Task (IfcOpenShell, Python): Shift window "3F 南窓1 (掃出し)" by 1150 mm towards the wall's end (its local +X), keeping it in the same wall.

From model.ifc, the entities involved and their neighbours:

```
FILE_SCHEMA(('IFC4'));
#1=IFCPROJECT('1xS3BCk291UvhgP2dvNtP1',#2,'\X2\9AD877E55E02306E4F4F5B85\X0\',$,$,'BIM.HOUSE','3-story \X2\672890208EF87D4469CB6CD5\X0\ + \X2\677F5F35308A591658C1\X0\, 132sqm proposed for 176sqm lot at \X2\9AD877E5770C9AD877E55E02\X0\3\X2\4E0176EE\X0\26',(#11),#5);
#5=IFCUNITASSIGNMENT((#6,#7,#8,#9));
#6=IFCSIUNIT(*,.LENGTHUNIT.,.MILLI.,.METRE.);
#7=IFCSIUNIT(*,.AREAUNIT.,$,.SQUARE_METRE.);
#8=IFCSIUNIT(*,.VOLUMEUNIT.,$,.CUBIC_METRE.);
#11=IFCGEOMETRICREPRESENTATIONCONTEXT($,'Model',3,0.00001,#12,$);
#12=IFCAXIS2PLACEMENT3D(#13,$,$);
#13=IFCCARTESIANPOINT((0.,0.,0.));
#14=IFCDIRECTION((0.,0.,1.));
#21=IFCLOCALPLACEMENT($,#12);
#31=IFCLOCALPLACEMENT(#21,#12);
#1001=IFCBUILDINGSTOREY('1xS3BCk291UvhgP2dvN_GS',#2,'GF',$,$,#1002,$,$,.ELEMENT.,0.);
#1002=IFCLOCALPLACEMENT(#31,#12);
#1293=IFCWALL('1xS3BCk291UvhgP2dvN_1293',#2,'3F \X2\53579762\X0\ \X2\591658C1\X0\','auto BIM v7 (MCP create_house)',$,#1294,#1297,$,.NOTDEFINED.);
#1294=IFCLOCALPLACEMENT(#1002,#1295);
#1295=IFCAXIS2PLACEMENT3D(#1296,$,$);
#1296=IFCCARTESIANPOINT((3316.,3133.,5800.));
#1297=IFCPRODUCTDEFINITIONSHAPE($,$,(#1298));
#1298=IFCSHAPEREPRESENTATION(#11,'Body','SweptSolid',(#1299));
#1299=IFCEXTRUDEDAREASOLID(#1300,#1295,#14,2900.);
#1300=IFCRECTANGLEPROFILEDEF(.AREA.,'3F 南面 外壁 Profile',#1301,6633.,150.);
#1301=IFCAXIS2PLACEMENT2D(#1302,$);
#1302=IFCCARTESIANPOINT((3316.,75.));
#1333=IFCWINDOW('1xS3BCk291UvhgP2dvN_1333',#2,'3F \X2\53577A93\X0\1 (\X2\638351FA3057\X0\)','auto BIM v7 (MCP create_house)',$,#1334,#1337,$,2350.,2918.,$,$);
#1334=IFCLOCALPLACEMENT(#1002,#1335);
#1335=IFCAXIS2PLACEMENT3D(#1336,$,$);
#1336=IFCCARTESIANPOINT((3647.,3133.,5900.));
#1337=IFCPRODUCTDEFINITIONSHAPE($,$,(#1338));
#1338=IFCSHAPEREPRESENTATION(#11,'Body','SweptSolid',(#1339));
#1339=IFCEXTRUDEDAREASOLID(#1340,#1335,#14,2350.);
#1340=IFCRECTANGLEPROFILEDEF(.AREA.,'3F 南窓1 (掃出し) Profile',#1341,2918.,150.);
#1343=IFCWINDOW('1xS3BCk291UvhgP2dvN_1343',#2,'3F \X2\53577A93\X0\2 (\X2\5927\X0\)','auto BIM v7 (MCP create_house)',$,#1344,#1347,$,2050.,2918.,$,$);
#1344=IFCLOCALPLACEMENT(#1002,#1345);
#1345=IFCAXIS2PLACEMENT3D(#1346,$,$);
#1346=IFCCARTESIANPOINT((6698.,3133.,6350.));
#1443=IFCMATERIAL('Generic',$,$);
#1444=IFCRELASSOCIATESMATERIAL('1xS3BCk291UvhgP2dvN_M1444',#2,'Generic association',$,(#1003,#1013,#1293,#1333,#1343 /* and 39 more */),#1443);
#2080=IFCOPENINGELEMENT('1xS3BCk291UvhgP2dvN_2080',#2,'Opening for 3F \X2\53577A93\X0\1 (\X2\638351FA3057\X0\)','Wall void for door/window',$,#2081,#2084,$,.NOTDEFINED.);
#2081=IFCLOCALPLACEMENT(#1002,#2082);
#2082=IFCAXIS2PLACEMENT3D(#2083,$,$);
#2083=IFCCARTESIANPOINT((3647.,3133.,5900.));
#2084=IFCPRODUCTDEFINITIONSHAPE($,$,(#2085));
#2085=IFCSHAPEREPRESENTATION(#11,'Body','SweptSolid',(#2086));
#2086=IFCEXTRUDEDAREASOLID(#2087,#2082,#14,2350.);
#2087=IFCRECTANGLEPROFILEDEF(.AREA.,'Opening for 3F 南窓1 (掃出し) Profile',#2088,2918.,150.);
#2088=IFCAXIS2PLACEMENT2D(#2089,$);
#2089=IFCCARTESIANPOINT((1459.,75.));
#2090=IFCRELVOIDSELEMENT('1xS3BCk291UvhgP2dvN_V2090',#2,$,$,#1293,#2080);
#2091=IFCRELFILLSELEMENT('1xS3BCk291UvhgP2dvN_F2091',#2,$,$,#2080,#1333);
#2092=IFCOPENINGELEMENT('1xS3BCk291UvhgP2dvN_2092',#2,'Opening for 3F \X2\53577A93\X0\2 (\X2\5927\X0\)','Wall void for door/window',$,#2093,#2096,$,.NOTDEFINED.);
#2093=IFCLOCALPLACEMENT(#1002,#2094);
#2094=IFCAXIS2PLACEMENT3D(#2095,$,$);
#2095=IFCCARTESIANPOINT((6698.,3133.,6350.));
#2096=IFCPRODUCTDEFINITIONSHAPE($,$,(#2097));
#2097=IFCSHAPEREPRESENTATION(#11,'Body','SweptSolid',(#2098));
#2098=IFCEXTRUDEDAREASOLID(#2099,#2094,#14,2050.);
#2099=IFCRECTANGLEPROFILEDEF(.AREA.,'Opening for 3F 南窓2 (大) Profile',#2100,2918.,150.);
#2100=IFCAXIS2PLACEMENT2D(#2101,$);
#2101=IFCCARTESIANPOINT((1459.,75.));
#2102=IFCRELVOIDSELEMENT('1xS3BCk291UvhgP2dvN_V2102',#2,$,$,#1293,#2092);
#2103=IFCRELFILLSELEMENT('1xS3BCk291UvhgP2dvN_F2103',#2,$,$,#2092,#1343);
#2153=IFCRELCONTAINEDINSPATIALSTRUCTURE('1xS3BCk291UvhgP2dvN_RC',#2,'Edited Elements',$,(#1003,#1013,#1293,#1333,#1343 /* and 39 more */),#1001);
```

```python
import ifcopenshell
import ifcopenshell.api.geometry
import ifcopenshell.util.placement
import ifcopenshell.util.unit

model = ifcopenshell.open("model.ifc")
unit_scale = ifcopenshell.util.unit.calculate_unit_scale(model)

window = model.by_guid("1xS3BCk291UvhgP2dvN_1333")
opening = window.FillsVoids[0].RelatingOpeningElement
wall = opening.VoidsElements[0].RelatingBuildingElement

wall_matrix = ifcopenshell.util.placement.get_local_placement(wall.ObjectPlacement)
shift = wall_matrix[:3, 0] * 1.15 / unit_scale
before = ifcopenshell.util.placement.get_local_placement(window.ObjectPlacement)[:3, 3].copy()

# The window is not placed relative to its opening, so move both.
for product in (opening, window):
    matrix = ifcopenshell.util.placement.get_local_placement(product.ObjectPlacement)
    matrix[:3, 3] += shift
    ifcopenshell.api.geometry.edit_object_placement(model, product=product, matrix=matrix, is_si=False)

after = ifcopenshell.util.placement.get_local_placement(window.ObjectPlacement)[:3, 3]
print("window moved by", (after - before).round(3) + 0.0)

model.write("model-out.ifc")
```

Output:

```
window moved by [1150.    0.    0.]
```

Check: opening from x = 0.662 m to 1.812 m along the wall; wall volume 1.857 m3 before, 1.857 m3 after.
